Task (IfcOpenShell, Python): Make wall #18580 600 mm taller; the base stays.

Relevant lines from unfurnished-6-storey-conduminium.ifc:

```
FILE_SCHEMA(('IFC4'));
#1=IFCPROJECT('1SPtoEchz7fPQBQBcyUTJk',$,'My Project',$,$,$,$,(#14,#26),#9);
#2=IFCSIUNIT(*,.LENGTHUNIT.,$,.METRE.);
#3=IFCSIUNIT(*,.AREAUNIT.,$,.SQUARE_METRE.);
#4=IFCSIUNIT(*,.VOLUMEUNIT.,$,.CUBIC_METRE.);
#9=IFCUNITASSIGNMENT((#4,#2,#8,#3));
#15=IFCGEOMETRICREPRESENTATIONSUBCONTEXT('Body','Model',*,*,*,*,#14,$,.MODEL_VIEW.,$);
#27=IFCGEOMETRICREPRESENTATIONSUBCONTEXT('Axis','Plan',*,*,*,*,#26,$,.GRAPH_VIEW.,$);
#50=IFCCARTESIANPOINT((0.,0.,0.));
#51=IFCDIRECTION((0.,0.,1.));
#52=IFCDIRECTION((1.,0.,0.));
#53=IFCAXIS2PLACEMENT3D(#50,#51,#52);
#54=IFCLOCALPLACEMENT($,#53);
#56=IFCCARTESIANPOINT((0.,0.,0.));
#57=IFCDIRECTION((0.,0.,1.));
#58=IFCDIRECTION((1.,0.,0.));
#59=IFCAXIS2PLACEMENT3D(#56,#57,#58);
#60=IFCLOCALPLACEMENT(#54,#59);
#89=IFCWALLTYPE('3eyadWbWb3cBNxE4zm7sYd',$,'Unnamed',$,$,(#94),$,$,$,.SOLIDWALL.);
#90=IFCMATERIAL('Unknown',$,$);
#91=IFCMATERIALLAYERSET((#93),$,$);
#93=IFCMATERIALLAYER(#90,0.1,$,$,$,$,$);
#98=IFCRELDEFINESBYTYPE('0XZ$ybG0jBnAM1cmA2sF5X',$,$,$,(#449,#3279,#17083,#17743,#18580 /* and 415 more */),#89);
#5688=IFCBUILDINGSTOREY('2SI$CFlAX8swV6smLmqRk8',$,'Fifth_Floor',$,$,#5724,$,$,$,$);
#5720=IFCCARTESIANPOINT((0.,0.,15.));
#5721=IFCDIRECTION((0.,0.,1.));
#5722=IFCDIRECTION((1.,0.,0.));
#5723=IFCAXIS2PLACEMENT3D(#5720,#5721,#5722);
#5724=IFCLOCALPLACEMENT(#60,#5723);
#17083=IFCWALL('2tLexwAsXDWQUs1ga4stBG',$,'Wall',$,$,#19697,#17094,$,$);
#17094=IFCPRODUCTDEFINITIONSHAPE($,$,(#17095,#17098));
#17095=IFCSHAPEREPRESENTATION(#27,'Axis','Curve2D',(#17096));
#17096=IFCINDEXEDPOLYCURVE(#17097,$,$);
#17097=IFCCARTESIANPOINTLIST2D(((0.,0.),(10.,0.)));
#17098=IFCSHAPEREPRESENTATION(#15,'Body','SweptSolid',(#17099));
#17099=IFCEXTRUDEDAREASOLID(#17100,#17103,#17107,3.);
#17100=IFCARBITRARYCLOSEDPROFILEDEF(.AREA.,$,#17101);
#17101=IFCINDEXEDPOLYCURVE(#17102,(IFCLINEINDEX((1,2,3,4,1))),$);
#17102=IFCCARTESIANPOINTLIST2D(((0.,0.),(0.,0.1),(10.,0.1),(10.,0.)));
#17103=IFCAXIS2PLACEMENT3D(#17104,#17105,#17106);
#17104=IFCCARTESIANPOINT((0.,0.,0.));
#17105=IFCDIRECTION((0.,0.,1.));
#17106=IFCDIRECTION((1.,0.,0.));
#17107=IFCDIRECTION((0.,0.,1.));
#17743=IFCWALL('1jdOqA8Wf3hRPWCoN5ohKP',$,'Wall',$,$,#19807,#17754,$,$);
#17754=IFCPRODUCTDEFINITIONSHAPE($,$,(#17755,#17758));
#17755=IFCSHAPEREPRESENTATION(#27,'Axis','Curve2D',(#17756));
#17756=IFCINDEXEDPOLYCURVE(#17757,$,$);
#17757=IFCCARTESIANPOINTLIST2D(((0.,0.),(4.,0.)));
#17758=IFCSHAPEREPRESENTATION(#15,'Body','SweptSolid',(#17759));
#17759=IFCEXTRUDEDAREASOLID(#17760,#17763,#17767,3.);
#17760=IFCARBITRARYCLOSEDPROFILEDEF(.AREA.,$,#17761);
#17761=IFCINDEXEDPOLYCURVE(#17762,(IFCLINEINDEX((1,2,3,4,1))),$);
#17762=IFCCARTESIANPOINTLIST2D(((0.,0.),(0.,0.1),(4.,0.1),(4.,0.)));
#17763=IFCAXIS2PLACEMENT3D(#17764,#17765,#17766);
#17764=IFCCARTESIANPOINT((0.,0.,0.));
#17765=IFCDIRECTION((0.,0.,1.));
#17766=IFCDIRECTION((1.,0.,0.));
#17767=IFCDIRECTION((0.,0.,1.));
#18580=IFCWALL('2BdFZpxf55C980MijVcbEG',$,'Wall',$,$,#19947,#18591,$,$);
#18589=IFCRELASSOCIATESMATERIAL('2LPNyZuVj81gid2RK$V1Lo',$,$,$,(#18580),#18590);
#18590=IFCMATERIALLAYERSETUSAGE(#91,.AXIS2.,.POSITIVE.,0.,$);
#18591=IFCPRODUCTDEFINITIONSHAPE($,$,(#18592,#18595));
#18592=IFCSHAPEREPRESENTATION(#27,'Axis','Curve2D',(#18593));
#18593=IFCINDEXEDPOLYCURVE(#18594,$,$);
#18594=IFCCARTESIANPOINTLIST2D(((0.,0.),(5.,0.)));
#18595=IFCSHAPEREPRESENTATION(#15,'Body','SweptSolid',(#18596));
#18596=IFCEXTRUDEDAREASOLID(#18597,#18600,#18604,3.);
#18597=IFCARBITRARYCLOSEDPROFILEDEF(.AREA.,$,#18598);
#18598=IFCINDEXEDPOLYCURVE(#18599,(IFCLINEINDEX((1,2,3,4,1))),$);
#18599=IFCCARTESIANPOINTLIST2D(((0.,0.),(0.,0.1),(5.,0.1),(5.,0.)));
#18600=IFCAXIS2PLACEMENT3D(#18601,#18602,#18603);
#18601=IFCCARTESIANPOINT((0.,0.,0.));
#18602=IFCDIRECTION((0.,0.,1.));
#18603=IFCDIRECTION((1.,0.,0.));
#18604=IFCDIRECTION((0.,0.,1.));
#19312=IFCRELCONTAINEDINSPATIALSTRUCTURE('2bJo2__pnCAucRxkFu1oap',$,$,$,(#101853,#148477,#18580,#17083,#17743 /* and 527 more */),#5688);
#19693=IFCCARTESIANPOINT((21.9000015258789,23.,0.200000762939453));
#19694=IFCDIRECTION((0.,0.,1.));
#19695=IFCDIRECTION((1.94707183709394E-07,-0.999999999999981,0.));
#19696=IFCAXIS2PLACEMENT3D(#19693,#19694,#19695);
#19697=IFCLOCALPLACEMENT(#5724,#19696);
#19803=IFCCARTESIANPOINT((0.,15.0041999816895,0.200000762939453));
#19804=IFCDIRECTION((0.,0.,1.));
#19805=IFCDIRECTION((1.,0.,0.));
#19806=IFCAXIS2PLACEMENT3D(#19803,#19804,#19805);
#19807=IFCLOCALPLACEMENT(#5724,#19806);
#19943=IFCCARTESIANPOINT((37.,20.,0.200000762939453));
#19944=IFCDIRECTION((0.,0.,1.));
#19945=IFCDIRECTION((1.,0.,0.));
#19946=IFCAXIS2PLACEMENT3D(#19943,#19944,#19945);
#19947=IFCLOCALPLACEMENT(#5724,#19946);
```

```python
import ifcopenshell
import ifcopenshell.geom
import ifcopenshell.util.representation
import ifcopenshell.util.shape

model = ifcopenshell.open("unfurnished-6-storey-conduminium.ifc")
settings = ifcopenshell.geom.settings()


def volume(element):
    """Net volume in cubic metres, openings subtracted."""
    shape = ifcopenshell.geom.create_shape(settings, element)
    return ifcopenshell.util.shape.get_volume(shape.geometry)


wall = model.by_id(18580)
before = volume(wall)

body = ifcopenshell.util.representation.get_representation(wall, "Model", "Body")
solid = body.Items[0]
old_height = solid.Depth
solid.Depth += 0.6
after = volume(wall)

print(f"height {old_height:g} -> {solid.Depth:g}, volume {before:.3f} -> {after:.3f} m3")

model.write("unfurnished-6-storey-conduminium_updated.ifc")
```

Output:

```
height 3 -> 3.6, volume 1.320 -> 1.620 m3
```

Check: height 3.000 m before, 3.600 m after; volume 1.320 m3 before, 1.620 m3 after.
